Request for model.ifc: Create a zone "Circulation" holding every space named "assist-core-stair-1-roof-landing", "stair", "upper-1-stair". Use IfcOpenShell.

First a look at what the model holds.

```python
import ifcopenshell

model = ifcopenshell.open("model.ifc")
print(model.schema)
seen = {}
for space in model.by_type("IfcSpace"):
    seen[space.LongName] = seen.get(space.LongName, 0) + 1
for name, count in sorted(seen.items(), key=str):
    print(count, "x", name)
print("zones:", [z.Name for z in model.by_type("IfcZone")][:20])
```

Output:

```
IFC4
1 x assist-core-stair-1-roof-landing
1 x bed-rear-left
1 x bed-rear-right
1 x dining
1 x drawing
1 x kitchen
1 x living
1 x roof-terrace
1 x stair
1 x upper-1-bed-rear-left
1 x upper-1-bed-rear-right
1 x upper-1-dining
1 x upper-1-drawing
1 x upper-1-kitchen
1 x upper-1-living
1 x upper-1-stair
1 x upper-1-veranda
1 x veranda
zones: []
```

```python
import ifcopenshell
import ifcopenshell.api.group
import ifcopenshell.api.root

model = ifcopenshell.open("model.ifc")

names = {"assist-core-stair-1-roof-landing", "stair", "upper-1-stair"}
spaces = [s for s in model.by_type("IfcSpace") if s.LongName in names]

zone = ifcopenshell.api.root.create_entity(model, ifc_class="IfcZone", name="Circulation")
ifcopenshell.api.group.assign_group(model, products=spaces, group=zone)
print(len(spaces), "spaces in", zone.Name)

model.write("model_rev.ifc")
```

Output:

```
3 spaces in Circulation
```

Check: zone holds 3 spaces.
